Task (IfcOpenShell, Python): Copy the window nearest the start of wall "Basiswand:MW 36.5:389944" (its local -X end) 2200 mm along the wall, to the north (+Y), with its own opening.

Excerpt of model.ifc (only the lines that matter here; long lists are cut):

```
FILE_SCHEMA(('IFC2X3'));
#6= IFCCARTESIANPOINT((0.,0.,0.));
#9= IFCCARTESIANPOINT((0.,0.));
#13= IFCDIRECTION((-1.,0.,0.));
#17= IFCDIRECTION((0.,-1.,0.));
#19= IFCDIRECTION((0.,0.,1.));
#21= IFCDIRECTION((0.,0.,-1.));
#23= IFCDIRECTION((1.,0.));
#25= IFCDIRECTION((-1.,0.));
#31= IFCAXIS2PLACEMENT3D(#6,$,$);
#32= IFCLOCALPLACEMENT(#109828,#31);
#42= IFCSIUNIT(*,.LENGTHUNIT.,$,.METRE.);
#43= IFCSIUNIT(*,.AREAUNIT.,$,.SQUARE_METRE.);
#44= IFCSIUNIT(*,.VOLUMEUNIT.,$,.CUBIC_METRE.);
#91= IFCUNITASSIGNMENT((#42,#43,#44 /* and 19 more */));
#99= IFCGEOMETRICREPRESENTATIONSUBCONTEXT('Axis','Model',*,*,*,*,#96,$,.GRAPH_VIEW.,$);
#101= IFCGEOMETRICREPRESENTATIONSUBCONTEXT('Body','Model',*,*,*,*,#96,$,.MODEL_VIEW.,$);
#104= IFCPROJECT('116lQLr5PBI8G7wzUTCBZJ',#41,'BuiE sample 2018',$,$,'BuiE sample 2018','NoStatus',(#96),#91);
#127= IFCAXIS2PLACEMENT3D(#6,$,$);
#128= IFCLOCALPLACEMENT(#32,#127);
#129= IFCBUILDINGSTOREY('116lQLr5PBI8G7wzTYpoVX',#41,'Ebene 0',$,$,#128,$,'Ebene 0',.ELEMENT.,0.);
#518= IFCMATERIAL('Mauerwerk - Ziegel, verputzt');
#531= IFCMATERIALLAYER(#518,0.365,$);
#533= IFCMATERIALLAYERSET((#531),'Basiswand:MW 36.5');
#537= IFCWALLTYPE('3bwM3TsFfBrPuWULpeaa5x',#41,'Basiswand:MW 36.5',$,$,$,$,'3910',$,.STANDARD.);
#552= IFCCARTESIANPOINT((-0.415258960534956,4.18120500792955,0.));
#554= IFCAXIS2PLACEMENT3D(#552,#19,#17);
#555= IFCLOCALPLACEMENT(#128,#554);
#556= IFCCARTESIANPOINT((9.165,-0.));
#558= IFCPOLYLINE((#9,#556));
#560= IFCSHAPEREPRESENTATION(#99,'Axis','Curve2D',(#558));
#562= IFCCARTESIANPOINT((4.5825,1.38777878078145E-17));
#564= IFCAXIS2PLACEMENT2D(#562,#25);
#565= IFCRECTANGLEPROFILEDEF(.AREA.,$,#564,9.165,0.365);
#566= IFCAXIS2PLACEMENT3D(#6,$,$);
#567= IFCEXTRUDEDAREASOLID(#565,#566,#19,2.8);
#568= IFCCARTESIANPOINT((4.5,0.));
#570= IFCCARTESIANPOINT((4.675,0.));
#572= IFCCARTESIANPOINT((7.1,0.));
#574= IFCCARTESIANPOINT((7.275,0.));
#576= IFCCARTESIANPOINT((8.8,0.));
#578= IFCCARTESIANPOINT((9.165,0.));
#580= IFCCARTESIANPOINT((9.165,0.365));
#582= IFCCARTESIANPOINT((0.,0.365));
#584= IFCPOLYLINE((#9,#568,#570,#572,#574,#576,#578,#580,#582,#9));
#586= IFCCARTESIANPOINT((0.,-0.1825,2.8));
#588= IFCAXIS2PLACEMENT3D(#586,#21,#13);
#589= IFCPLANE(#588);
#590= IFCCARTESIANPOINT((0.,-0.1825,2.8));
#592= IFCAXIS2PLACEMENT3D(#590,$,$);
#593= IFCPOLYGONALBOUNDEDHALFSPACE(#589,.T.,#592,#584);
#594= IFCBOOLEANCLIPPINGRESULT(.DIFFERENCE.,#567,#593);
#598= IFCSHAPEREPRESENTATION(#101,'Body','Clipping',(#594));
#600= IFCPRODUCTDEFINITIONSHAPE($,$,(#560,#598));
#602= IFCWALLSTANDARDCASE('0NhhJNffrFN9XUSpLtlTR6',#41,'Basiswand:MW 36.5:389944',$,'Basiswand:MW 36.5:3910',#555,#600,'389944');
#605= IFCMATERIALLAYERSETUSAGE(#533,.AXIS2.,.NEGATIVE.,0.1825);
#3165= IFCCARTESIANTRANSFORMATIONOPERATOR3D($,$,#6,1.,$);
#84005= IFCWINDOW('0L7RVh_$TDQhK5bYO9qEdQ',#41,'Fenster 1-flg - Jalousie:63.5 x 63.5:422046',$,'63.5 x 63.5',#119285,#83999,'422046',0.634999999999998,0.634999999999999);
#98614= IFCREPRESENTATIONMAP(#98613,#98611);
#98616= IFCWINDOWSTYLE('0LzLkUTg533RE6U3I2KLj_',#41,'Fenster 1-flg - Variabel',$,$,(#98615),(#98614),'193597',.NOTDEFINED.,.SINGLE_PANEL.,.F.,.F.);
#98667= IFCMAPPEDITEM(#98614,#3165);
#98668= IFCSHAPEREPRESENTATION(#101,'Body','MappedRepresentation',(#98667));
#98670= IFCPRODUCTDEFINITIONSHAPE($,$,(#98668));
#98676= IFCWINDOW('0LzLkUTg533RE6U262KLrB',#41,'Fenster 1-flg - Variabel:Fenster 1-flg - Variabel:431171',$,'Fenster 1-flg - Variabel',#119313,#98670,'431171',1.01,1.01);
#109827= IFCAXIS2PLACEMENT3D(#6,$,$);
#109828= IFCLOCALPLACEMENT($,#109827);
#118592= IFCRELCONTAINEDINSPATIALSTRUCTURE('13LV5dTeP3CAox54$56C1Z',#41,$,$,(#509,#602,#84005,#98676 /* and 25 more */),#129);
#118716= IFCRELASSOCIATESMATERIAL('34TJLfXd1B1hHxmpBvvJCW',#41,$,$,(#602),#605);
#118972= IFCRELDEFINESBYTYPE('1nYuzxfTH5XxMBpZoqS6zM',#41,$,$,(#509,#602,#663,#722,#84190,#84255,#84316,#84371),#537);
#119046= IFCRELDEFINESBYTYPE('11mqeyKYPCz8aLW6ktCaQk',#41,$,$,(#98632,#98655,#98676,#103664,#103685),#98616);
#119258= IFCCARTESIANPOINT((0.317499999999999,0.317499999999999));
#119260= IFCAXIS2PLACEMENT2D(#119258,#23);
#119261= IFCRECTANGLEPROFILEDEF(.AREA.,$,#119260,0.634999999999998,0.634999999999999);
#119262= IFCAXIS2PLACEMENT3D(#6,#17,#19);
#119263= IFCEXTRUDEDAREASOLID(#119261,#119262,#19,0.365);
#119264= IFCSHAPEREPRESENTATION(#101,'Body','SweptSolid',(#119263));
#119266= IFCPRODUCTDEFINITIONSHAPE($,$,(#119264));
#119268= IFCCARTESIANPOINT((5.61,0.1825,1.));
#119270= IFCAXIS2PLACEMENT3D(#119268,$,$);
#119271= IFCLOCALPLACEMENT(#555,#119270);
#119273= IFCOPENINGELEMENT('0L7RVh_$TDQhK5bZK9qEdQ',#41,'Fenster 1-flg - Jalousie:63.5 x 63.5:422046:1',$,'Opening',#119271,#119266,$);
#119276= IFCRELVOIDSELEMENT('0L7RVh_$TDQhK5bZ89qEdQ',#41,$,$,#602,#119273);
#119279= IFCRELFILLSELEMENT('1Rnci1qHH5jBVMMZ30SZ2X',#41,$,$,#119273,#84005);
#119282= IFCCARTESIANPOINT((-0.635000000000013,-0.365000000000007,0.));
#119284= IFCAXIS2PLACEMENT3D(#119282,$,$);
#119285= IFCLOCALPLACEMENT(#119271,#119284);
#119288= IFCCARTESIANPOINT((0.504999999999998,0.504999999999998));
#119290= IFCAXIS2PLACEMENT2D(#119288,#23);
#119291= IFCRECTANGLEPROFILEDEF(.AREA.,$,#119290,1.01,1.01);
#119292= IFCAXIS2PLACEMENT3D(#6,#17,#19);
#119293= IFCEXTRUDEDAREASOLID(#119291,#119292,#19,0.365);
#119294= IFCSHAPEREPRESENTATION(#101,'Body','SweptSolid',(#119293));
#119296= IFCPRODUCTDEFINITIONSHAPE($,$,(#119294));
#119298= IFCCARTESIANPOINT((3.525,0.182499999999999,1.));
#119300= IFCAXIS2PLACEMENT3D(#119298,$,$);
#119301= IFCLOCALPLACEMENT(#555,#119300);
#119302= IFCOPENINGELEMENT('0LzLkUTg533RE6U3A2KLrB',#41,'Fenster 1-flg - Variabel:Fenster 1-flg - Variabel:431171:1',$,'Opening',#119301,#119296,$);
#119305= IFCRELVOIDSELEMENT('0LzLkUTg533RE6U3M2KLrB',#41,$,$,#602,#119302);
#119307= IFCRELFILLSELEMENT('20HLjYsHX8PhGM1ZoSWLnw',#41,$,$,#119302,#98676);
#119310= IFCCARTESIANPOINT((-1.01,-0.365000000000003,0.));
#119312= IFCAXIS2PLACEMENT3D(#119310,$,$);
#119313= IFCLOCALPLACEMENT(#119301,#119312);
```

```python
import ifcopenshell
import ifcopenshell.api.feature
import ifcopenshell.api.geometry
import ifcopenshell.api.root
import ifcopenshell.geom
import ifcopenshell.util.element
import ifcopenshell.util.placement
import ifcopenshell.util.shape
import ifcopenshell.util.unit

model = ifcopenshell.open("model.ifc")
unit_scale = ifcopenshell.util.unit.calculate_unit_scale(model)
settings = ifcopenshell.geom.settings()


def volume(element):
    """Net volume in cubic metres, openings subtracted."""
    shape = ifcopenshell.geom.create_shape(settings, element)
    return ifcopenshell.util.shape.get_volume(shape.geometry)


def reuse_history(source, copy):
    """copy_class also copies each property set's owner history, people and application; keep the originals."""
    for rel in copy.IsDefinedBy:
        if rel.is_a("IfcRelDefinesByProperties") and (history := rel.RelatingPropertyDefinition.OwnerHistory):
            rel.RelatingPropertyDefinition.OwnerHistory = source.OwnerHistory
            ifcopenshell.util.element.remove_deep2(model, history)


window = model.by_guid("0LzLkUTg533RE6U262KLrB")
opening = window.FillsVoids[0].RelatingOpeningElement
wall = opening.VoidsElements[0].RelatingBuildingElement
before = volume(wall)
shift = ifcopenshell.util.placement.get_local_placement(wall.ObjectPlacement)[:3, 0] * -2.2 / unit_scale

# copy_class copies the void relationship, type, container and properties, but no geometry.
new_opening = ifcopenshell.api.root.copy_class(model, product=opening)
new_opening.Representation = ifcopenshell.util.element.copy_deep(
    model, opening.Representation, exclude=["IfcGeometricRepresentationContext", "IfcRepresentationMap"]
)
new_opening.Name = "Fenster 1-flg - Variabel:Fenster 1-flg - Variabel"
new_window = ifcopenshell.api.root.copy_class(model, product=window)
new_window.Representation = ifcopenshell.util.element.copy_deep(
    model, window.Representation, exclude=["IfcGeometricRepresentationContext", "IfcRepresentationMap"]
)
new_window.Name = "Fenster 1-flg - Variabel:Fenster 1-flg - Variabel"
new_window.Tag = None
reuse_history(window, new_window)
fills = ifcopenshell.api.feature.add_filling(model, opening=new_opening, element=new_window)
fills.OwnerHistory = new_window.OwnerHistory  # required in IFC2X3

for old, new in ((opening, new_opening), (window, new_window)):
    matrix = ifcopenshell.util.placement.get_local_placement(old.ObjectPlacement)
    matrix[:3, 3] += shift
    ifcopenshell.api.geometry.edit_object_placement(model, product=new, matrix=matrix, is_si=False)

after = volume(wall)

print(f"wall volume {before:.3f} -> {after:.3f} m3")

model.write("model_rev.ifc")
```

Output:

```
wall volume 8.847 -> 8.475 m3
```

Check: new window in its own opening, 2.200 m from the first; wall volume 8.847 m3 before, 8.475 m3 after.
